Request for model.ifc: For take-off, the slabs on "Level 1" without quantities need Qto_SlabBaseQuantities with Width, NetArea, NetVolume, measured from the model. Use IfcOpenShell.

First a look at what the model holds.

```python
import ifcopenshell
import ifcopenshell.util.element
import ifcopenshell.util.unit

model = ifcopenshell.open("model.ifc")
print(model.schema)
for unit_type in ("LENGTHUNIT", "AREAUNIT", "VOLUMEUNIT"):
    print(unit_type, ifcopenshell.util.unit.calculate_unit_scale(model, unit_type))
storey = next(s for s in model.by_type("IfcBuildingStorey") if s.Name == "Level 1")
slabs = [e for e in ifcopenshell.util.element.get_decomposition(storey) if e.is_a("IfcSlab")]
for e in sorted(slabs, key=lambda e: e.id()):
    print(e.id(), e.is_a(), e.Name, list(ifcopenshell.util.element.get_psets(e, qtos_only=True)), sep=" | ")
```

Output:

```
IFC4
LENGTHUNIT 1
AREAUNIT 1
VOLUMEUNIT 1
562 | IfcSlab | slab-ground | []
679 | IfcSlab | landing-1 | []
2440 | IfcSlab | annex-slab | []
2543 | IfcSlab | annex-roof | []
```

```python
import ifcopenshell
import ifcopenshell.api.pset
import ifcopenshell.geom
import ifcopenshell.util.element
import ifcopenshell.util.shape
import ifcopenshell.util.unit

model = ifcopenshell.open("model.ifc")
unit_scale = ifcopenshell.util.unit.calculate_unit_scale(model)
area_scale = ifcopenshell.util.unit.calculate_unit_scale(model, "AREAUNIT")
volume_scale = ifcopenshell.util.unit.calculate_unit_scale(model, "VOLUMEUNIT")
settings = ifcopenshell.geom.settings()

storey = next(s for s in model.by_type("IfcBuildingStorey") if s.Name == "Level 1")
slabs = [e for e in ifcopenshell.util.element.get_decomposition(storey) if e.is_a("IfcSlab")]

for e in sorted(slabs, key=lambda e: e.id()):
    if ifcopenshell.util.element.get_psets(e, qtos_only=True, should_inherit=False):
        continue
    # Geometry comes back in metres, in the element's own axes.
    shape = ifcopenshell.geom.create_shape(settings, e)
    values = {
        "Width": ifcopenshell.util.shape.get_z(shape.geometry) / unit_scale,
        "NetArea": ifcopenshell.util.shape.get_footprint_area(shape.geometry) / area_scale,
        "NetVolume": ifcopenshell.util.shape.get_volume(shape.geometry) / volume_scale,
    }
    qto = ifcopenshell.api.pset.add_qto(model, product=e, name="Qto_SlabBaseQuantities")
    ifcopenshell.api.pset.edit_qto(model, qto=qto, properties=values)
    print(e.id(), {k: round(v, 3) for k, v in values.items()})

model.write("model_rev.ifc")
```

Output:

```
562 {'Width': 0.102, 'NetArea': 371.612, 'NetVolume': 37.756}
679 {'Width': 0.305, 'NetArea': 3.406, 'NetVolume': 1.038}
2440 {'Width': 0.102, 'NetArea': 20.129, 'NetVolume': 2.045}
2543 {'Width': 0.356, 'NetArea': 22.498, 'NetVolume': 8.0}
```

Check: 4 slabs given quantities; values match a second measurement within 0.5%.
